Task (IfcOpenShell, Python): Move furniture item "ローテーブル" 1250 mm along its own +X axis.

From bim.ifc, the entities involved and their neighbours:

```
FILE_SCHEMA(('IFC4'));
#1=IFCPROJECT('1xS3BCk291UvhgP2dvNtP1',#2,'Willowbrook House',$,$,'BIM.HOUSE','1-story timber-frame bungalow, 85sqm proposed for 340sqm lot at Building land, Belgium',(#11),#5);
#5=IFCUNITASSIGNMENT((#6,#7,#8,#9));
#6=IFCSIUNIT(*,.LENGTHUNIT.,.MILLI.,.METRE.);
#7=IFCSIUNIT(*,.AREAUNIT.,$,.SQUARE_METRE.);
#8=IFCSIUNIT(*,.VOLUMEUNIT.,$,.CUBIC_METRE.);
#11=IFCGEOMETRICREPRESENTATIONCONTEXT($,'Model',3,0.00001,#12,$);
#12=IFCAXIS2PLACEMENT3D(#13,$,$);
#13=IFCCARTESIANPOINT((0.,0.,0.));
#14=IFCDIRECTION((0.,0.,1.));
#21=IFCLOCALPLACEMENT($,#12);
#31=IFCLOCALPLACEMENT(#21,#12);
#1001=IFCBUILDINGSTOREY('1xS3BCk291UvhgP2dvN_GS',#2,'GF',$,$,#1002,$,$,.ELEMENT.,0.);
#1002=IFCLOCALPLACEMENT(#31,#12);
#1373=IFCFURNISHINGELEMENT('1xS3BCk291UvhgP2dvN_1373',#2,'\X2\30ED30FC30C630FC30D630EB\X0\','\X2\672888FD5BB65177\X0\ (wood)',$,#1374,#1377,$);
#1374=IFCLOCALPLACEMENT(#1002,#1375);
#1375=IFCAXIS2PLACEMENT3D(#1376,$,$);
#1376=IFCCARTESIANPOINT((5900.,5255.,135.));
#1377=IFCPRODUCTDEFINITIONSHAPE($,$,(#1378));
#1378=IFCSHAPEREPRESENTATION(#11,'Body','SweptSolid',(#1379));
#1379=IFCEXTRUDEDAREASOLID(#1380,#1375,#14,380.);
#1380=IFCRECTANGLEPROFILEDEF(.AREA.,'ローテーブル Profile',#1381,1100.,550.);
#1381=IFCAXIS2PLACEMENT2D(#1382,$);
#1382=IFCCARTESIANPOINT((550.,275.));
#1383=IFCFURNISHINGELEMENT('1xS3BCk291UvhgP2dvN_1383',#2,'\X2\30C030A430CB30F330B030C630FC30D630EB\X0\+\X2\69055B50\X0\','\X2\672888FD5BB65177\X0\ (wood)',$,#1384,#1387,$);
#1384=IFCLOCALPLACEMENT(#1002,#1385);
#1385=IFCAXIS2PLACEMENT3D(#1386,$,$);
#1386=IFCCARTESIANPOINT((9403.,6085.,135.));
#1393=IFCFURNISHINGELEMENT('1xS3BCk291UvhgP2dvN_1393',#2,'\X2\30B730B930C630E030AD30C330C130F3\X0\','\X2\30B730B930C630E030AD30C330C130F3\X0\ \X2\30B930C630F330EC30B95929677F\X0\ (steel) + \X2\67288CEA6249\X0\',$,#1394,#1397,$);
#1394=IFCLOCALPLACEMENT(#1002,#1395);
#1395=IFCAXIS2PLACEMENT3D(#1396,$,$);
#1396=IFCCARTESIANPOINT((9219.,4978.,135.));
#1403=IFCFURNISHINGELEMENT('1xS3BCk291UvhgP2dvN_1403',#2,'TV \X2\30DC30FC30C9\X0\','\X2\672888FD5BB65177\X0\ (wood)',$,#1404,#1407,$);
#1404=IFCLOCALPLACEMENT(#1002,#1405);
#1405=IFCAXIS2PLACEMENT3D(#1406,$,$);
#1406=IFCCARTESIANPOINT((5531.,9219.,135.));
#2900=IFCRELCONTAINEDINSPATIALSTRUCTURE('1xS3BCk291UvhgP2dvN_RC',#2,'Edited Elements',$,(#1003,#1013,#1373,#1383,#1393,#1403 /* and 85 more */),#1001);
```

```python
import ifcopenshell
import ifcopenshell.api.geometry
import ifcopenshell.util.placement

model = ifcopenshell.open("bim.ifc")

item = model.by_guid("1xS3BCk291UvhgP2dvN_1373")
matrix = ifcopenshell.util.placement.get_local_placement(item.ObjectPlacement)
matrix[:3, 3] += matrix[:3, 0] * 1250.0
ifcopenshell.api.geometry.edit_object_placement(model, product=item, matrix=matrix, is_si=False)

print(ifcopenshell.util.placement.get_local_placement(item.ObjectPlacement).round(3) + 0.0)

model.write("bim-out.ifc")
```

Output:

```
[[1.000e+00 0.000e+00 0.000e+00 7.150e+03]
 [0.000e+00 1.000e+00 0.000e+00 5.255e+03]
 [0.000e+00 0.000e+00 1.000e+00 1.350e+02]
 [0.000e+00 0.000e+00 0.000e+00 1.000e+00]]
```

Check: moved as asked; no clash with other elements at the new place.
